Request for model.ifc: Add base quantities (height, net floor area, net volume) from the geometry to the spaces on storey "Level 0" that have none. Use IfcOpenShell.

First a look at what the model holds.

```python
import ifcopenshell
import ifcopenshell.util.element
import ifcopenshell.util.unit

model = ifcopenshell.open("model.ifc")
print(model.schema)
for unit_type in ("LENGTHUNIT", "AREAUNIT", "VOLUMEUNIT"):
    print(unit_type, ifcopenshell.util.unit.calculate_unit_scale(model, unit_type))
storey = next(s for s in model.by_type("IfcBuildingStorey") if s.Name == "Level 0")
spaces = [e for e in ifcopenshell.util.element.get_decomposition(storey) if e.is_a("IfcSpace")]
for e in sorted(spaces, key=lambda e: e.id()):
    print(e.id(), e.is_a(), e.Name, list(ifcopenshell.util.element.get_psets(e, qtos_only=True)), sep=" | ")
```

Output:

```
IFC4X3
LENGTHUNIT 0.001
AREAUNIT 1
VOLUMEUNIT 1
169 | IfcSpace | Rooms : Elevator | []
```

```python
import ifcopenshell
import ifcopenshell.api.pset
import ifcopenshell.geom
import ifcopenshell.util.element
import ifcopenshell.util.shape
import ifcopenshell.util.unit

model = ifcopenshell.open("model.ifc")
unit_scale = ifcopenshell.util.unit.calculate_unit_scale(model)
area_scale = ifcopenshell.util.unit.calculate_unit_scale(model, "AREAUNIT")
volume_scale = ifcopenshell.util.unit.calculate_unit_scale(model, "VOLUMEUNIT")
settings = ifcopenshell.geom.settings()

storey = next(s for s in model.by_type("IfcBuildingStorey") if s.Name == "Level 0")
spaces = [e for e in ifcopenshell.util.element.get_decomposition(storey) if e.is_a("IfcSpace")]

for e in sorted(spaces, key=lambda e: e.id()):
    if ifcopenshell.util.element.get_psets(e, qtos_only=True, should_inherit=False):
        continue
    # Geometry comes back in metres, in the element's own axes.
    shape = ifcopenshell.geom.create_shape(settings, e)
    values = {
        "Height": ifcopenshell.util.shape.get_z(shape.geometry) / unit_scale,
        "NetFloorArea": ifcopenshell.util.shape.get_footprint_area(shape.geometry) / area_scale,
        "NetVolume": ifcopenshell.util.shape.get_volume(shape.geometry) / volume_scale,
    }
    qto = ifcopenshell.api.pset.add_qto(model, product=e, name="Qto_SpaceBaseQuantities")
    ifcopenshell.api.pset.edit_qto(model, qto=qto, properties=values)
    print(e.id(), {k: round(v, 3) for k, v in values.items()})

model.write("model_updated.ifc")
```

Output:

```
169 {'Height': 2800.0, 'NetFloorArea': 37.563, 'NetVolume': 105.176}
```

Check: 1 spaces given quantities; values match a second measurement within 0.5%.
